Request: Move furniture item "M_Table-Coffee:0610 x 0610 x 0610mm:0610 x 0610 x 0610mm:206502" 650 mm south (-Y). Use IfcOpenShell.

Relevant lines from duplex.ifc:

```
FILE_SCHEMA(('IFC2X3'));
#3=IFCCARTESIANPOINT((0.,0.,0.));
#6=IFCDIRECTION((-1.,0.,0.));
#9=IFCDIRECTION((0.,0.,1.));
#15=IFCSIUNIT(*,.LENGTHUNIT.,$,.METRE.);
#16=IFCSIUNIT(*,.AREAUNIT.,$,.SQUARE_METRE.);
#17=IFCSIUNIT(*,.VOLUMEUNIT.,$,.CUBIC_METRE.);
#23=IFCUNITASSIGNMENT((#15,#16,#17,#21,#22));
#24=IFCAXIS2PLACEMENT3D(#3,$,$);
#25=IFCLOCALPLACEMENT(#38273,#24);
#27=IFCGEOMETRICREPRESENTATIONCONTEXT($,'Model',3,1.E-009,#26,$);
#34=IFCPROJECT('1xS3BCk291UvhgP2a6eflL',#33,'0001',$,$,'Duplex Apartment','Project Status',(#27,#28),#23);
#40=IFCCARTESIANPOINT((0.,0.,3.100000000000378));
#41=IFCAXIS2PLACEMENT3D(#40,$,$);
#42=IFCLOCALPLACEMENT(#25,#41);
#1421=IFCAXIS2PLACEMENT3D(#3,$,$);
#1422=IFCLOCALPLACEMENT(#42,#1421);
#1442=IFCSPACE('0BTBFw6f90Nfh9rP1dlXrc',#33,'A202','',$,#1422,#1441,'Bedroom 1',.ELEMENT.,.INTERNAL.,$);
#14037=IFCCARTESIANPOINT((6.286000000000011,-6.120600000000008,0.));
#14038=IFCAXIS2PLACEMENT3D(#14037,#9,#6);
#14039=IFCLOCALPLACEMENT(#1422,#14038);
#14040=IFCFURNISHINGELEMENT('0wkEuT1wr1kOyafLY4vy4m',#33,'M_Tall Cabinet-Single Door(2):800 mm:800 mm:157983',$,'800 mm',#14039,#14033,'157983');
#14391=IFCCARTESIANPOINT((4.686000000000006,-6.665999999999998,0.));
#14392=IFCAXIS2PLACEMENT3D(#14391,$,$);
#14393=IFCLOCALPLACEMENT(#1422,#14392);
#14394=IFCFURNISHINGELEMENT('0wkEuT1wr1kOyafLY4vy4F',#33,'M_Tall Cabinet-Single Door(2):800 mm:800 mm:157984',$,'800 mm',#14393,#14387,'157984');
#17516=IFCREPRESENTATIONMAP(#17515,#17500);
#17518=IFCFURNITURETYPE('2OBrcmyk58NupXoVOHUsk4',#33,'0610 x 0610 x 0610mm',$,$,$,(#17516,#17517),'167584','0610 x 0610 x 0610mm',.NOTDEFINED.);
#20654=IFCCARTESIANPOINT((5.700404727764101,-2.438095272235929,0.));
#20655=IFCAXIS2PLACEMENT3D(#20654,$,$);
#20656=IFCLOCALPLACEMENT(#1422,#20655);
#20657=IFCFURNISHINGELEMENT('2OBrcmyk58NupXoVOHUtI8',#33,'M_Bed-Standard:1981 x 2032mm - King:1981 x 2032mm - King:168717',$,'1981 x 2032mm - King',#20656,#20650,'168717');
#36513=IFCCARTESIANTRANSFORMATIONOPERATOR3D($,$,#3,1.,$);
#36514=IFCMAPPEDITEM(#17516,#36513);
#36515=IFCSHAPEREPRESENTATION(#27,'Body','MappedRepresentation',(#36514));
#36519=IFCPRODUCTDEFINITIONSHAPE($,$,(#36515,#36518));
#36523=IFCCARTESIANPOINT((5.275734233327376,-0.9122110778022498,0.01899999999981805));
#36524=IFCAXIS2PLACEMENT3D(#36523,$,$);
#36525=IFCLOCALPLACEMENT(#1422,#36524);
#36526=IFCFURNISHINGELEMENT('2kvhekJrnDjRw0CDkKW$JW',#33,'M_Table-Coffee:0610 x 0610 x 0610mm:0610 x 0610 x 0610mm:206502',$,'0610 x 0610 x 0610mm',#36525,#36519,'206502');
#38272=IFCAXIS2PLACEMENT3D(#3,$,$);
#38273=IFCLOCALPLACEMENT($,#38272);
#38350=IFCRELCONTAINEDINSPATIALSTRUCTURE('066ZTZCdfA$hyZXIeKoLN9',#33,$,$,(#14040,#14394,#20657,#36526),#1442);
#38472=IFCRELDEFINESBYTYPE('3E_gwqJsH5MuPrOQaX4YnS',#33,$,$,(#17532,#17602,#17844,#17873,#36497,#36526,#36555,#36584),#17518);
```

```python
import ifcopenshell
import ifcopenshell.api.geometry
import ifcopenshell.util.placement

model = ifcopenshell.open("duplex.ifc")

item = model.by_id(36526)
matrix = ifcopenshell.util.placement.get_local_placement(item.ObjectPlacement)
matrix[1, 3] -= 0.65
ifcopenshell.api.geometry.edit_object_placement(model, product=item, matrix=matrix, is_si=False)

print(ifcopenshell.util.placement.get_local_placement(item.ObjectPlacement).round(3) + 0.0)

model.write("duplex_rev.ifc")
```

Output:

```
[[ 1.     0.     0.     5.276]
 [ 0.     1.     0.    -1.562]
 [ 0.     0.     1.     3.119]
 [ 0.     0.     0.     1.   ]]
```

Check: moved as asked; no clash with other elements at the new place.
